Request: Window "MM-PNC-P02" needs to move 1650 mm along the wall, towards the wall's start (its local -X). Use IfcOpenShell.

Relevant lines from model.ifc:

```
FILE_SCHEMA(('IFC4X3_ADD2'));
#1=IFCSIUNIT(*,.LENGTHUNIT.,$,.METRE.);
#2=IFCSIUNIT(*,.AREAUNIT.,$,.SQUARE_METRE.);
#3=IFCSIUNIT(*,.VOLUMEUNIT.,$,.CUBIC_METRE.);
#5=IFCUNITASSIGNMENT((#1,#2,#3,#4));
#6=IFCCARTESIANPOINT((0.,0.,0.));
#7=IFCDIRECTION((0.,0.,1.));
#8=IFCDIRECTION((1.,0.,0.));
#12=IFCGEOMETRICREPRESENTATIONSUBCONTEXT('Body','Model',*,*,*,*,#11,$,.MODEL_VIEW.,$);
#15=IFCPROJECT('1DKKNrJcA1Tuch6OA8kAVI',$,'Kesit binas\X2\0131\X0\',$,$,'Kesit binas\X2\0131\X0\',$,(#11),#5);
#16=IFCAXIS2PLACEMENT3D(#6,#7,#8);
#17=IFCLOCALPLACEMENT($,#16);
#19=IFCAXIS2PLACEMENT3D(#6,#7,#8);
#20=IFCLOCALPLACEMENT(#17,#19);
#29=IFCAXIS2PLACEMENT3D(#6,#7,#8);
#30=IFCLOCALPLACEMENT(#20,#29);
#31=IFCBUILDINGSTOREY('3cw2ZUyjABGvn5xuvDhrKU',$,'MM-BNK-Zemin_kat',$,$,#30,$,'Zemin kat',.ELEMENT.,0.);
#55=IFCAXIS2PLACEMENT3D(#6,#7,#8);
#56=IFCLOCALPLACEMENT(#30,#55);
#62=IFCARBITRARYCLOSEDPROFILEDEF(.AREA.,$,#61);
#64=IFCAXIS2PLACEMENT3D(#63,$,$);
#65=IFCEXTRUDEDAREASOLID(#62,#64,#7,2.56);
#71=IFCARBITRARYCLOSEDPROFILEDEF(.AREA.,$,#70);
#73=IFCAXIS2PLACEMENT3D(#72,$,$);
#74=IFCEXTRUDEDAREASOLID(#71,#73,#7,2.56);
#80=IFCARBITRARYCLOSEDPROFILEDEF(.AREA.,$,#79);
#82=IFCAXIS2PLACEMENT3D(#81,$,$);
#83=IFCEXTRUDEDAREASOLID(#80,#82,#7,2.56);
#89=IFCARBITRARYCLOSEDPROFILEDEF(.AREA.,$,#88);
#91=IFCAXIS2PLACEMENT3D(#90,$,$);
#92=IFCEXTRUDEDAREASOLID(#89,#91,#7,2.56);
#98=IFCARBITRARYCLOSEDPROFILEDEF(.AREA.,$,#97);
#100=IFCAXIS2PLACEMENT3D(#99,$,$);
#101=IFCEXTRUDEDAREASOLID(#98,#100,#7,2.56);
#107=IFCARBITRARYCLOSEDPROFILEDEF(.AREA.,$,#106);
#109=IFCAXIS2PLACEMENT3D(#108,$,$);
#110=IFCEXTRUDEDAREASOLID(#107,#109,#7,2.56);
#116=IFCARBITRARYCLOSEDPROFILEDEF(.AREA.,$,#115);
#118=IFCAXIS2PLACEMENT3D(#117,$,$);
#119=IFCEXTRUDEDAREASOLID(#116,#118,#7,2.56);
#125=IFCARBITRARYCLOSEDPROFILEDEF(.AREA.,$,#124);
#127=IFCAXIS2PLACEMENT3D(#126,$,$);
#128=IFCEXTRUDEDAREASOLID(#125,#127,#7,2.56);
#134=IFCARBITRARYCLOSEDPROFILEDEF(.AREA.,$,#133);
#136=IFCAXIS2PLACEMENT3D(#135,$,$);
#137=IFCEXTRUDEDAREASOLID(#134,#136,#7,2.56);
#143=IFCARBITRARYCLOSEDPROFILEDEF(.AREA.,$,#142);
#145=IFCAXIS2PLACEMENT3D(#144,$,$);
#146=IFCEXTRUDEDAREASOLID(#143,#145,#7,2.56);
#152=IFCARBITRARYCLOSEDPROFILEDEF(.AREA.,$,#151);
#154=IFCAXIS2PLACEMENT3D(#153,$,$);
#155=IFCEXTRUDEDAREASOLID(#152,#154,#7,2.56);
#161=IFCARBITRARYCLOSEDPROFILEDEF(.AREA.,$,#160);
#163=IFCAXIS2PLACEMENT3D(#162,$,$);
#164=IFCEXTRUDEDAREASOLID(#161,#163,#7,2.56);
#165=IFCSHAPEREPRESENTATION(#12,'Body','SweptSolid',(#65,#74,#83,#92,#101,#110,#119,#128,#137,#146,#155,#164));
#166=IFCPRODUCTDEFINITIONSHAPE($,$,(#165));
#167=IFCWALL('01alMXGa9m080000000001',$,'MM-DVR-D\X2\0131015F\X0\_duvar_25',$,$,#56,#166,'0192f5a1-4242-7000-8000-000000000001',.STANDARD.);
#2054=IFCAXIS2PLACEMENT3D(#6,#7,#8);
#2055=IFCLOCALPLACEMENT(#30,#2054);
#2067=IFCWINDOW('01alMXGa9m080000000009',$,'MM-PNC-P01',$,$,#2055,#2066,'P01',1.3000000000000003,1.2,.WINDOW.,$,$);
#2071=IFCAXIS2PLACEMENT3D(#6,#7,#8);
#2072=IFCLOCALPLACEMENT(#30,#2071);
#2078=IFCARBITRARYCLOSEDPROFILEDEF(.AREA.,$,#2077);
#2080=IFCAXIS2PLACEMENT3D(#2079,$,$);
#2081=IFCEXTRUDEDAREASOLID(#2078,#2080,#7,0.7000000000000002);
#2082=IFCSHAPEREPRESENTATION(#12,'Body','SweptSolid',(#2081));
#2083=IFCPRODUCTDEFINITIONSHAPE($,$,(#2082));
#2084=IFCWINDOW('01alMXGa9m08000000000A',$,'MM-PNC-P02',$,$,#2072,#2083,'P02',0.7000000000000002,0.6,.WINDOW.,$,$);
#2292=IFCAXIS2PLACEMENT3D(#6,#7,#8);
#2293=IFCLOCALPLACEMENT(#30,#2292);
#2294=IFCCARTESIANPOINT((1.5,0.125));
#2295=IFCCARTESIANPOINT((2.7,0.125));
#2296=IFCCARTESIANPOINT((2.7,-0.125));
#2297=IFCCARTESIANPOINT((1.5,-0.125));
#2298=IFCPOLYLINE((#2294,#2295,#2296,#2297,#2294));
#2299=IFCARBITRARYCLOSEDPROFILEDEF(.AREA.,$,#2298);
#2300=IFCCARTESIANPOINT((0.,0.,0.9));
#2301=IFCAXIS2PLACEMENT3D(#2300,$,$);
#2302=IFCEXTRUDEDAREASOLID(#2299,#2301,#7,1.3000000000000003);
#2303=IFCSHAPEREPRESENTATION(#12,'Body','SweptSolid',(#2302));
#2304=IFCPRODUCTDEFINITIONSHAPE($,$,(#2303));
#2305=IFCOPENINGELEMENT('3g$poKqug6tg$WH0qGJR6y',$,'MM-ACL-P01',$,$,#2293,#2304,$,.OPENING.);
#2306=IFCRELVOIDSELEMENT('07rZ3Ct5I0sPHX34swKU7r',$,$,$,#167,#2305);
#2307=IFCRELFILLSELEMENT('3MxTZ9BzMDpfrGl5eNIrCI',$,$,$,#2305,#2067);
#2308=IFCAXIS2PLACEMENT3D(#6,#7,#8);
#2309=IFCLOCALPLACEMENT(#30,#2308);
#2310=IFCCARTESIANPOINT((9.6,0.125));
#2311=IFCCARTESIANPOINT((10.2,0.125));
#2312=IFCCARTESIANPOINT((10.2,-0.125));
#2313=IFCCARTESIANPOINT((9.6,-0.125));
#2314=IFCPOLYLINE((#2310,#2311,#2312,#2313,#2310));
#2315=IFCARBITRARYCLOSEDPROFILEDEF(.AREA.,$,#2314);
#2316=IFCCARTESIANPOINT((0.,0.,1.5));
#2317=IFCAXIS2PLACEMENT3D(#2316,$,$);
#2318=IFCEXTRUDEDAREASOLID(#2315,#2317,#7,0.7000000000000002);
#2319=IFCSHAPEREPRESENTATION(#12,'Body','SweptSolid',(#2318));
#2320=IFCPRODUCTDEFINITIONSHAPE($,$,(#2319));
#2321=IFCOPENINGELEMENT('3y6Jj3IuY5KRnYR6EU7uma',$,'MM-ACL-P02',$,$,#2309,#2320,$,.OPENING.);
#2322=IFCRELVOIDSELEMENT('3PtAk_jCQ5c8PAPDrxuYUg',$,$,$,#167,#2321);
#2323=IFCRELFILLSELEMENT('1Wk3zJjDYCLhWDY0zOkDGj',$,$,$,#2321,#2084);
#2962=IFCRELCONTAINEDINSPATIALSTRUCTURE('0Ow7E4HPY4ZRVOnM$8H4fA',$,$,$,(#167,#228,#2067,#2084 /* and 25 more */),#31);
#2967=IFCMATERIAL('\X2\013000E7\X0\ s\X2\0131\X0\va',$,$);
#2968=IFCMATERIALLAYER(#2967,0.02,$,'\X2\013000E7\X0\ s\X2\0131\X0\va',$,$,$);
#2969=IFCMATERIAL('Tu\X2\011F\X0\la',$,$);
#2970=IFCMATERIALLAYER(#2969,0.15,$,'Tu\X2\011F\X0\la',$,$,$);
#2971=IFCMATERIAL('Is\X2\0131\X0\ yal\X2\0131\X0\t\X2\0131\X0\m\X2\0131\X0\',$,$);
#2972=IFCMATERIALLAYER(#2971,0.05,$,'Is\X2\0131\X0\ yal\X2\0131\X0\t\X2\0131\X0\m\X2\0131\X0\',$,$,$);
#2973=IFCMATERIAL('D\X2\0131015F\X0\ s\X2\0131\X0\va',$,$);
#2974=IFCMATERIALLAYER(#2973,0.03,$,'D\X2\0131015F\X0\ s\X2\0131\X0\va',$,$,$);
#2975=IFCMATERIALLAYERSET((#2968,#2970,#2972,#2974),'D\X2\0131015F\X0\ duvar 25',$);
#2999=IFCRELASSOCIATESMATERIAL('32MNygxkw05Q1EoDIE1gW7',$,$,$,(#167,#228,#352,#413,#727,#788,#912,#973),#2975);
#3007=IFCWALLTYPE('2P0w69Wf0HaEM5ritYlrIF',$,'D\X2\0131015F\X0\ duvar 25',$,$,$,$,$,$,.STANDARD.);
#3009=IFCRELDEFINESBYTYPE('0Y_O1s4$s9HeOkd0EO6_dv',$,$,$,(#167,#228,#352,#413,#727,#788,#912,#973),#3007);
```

```python
import ifcopenshell
import ifcopenshell.api.geometry
import ifcopenshell.util.placement
import ifcopenshell.util.unit

model = ifcopenshell.open("model.ifc")
unit_scale = ifcopenshell.util.unit.calculate_unit_scale(model)

window = model.by_guid("01alMXGa9m08000000000A")
opening = window.FillsVoids[0].RelatingOpeningElement
wall = opening.VoidsElements[0].RelatingBuildingElement

wall_matrix = ifcopenshell.util.placement.get_local_placement(wall.ObjectPlacement)
shift = wall_matrix[:3, 0] * -1.65 / unit_scale
before = ifcopenshell.util.placement.get_local_placement(window.ObjectPlacement)[:3, 3].copy()

# The window is not placed relative to its opening, so move both.
for product in (opening, window):
    matrix = ifcopenshell.util.placement.get_local_placement(product.ObjectPlacement)
    matrix[:3, 3] += shift
    ifcopenshell.api.geometry.edit_object_placement(model, product=product, matrix=matrix, is_si=False)

after = ifcopenshell.util.placement.get_local_placement(window.ObjectPlacement)[:3, 3]
print("window moved by", (after - before).round(3) + 0.0)

model.write("model_v2.ifc")
```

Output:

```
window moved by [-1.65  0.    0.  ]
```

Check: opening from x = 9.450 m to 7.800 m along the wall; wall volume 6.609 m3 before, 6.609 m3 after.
